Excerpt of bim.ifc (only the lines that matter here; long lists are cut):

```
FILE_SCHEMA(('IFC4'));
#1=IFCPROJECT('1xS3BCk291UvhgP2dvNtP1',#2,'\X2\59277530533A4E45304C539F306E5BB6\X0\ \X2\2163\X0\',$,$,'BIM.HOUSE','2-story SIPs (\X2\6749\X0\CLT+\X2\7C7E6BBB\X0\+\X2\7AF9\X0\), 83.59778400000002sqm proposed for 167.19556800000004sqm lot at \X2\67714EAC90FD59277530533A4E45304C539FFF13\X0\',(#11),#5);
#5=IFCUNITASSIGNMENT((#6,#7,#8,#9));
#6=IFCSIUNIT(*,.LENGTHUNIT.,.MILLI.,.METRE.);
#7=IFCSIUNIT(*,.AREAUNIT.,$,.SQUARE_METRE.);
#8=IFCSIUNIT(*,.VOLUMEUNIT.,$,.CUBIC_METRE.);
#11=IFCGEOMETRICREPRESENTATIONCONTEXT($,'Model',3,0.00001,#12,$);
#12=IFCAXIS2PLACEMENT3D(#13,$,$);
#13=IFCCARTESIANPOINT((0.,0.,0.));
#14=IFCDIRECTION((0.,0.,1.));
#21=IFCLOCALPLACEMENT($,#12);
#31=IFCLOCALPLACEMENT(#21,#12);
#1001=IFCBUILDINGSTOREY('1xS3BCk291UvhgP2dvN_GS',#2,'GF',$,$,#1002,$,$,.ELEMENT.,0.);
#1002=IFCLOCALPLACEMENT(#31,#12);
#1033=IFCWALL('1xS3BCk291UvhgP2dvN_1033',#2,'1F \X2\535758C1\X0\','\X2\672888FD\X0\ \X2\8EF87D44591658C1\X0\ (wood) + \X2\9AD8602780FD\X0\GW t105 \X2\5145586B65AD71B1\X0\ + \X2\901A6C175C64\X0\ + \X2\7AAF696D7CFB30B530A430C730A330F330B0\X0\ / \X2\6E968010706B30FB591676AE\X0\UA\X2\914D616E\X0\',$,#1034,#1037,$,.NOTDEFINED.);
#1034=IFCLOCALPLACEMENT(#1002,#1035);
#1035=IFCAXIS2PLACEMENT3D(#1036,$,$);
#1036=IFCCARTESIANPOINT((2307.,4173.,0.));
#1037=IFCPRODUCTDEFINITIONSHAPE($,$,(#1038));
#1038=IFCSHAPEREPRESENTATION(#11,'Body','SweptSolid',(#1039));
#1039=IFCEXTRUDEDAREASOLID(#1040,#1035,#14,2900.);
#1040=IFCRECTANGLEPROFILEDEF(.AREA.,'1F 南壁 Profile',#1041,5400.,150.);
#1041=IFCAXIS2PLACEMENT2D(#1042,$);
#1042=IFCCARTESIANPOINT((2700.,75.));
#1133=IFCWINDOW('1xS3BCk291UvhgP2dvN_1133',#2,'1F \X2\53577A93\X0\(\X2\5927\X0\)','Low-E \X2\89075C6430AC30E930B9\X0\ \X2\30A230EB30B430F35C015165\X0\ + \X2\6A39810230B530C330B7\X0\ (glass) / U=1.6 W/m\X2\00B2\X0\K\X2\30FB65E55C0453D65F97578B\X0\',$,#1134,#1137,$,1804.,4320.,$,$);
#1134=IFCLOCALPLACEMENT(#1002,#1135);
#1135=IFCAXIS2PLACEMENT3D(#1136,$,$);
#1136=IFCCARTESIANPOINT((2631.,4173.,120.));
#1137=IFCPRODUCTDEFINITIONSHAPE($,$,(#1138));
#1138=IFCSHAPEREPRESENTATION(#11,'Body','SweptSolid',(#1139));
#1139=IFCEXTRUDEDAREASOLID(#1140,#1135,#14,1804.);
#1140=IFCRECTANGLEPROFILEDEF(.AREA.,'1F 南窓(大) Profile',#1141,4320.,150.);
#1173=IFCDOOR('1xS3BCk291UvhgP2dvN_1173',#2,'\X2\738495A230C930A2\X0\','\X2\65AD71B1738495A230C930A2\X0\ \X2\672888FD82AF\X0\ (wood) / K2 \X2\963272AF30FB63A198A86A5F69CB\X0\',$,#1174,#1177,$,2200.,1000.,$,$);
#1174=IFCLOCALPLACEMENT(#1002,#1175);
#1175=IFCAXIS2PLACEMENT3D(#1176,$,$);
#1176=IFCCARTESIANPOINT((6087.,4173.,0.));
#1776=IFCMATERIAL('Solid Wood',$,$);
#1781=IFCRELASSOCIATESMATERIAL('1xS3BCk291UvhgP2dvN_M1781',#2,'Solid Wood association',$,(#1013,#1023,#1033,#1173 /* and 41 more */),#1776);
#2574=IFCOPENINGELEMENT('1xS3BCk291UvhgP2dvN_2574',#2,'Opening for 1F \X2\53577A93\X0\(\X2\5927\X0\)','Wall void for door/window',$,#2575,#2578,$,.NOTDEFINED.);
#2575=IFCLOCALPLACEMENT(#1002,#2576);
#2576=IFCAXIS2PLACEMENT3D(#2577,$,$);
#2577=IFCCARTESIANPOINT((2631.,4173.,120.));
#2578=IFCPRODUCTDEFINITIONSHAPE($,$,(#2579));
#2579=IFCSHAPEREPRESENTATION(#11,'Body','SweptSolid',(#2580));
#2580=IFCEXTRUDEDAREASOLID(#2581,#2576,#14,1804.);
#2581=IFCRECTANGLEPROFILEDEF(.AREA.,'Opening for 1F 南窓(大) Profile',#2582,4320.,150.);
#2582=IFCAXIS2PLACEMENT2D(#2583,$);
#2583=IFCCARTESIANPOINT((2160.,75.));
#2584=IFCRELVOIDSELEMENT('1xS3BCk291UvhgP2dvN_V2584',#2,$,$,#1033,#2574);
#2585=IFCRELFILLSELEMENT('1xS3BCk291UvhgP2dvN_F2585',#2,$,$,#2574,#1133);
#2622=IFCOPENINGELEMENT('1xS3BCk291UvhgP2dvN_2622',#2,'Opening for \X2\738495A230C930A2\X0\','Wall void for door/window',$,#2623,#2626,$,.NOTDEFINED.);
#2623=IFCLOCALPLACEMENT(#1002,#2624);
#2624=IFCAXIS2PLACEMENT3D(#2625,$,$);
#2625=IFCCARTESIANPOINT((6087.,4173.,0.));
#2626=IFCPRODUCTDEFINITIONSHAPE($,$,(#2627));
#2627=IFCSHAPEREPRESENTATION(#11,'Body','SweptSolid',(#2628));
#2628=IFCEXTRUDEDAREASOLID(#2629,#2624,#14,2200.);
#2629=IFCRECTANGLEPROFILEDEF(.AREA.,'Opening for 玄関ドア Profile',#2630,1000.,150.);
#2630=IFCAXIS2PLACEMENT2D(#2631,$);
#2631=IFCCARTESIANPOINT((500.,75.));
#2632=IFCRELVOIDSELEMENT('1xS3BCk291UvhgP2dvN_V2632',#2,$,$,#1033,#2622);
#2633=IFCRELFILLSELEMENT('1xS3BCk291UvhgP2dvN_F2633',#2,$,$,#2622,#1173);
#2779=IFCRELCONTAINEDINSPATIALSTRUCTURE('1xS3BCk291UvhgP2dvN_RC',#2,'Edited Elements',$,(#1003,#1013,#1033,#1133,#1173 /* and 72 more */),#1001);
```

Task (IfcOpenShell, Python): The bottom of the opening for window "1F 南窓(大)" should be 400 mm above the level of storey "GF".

```python
import numpy as np
import ifcopenshell
import ifcopenshell.api.geometry
import ifcopenshell.geom
import ifcopenshell.util.element
import ifcopenshell.util.placement
import ifcopenshell.util.shape
import ifcopenshell.util.unit

model = ifcopenshell.open("bim.ifc")
unit_scale = ifcopenshell.util.unit.calculate_unit_scale(model)

window = model.by_guid("1xS3BCk291UvhgP2dvN_1133")
opening = window.FillsVoids[0].RelatingOpeningElement
storey = ifcopenshell.util.element.get_container(window, ifc_class="IfcBuildingStorey")
level = ifcopenshell.util.placement.get_local_placement(storey.ObjectPlacement)[2, 3]

# The opening's origin need not be at the sill, so measure its lowest point.
shape = ifcopenshell.geom.create_shape(ifcopenshell.geom.settings(), opening)
bottom = ifcopenshell.util.shape.get_shape_bottom_elevation(shape, shape.geometry) / unit_scale
dz = level + 0.4 / unit_scale - bottom

shift = np.array([0.0, 0.0, dz])
# The window is not placed relative to its opening, so move both.
for product in (opening, window):
    matrix = ifcopenshell.util.placement.get_local_placement(product.ObjectPlacement)
    matrix[:3, 3] += shift
    ifcopenshell.api.geometry.edit_object_placement(model, product=product, matrix=matrix, is_si=False)

print(f"moved by {dz * unit_scale:+.3f} m")

model.write("bim-out.ifc")
```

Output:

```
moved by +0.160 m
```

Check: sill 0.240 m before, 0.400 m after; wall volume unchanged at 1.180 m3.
